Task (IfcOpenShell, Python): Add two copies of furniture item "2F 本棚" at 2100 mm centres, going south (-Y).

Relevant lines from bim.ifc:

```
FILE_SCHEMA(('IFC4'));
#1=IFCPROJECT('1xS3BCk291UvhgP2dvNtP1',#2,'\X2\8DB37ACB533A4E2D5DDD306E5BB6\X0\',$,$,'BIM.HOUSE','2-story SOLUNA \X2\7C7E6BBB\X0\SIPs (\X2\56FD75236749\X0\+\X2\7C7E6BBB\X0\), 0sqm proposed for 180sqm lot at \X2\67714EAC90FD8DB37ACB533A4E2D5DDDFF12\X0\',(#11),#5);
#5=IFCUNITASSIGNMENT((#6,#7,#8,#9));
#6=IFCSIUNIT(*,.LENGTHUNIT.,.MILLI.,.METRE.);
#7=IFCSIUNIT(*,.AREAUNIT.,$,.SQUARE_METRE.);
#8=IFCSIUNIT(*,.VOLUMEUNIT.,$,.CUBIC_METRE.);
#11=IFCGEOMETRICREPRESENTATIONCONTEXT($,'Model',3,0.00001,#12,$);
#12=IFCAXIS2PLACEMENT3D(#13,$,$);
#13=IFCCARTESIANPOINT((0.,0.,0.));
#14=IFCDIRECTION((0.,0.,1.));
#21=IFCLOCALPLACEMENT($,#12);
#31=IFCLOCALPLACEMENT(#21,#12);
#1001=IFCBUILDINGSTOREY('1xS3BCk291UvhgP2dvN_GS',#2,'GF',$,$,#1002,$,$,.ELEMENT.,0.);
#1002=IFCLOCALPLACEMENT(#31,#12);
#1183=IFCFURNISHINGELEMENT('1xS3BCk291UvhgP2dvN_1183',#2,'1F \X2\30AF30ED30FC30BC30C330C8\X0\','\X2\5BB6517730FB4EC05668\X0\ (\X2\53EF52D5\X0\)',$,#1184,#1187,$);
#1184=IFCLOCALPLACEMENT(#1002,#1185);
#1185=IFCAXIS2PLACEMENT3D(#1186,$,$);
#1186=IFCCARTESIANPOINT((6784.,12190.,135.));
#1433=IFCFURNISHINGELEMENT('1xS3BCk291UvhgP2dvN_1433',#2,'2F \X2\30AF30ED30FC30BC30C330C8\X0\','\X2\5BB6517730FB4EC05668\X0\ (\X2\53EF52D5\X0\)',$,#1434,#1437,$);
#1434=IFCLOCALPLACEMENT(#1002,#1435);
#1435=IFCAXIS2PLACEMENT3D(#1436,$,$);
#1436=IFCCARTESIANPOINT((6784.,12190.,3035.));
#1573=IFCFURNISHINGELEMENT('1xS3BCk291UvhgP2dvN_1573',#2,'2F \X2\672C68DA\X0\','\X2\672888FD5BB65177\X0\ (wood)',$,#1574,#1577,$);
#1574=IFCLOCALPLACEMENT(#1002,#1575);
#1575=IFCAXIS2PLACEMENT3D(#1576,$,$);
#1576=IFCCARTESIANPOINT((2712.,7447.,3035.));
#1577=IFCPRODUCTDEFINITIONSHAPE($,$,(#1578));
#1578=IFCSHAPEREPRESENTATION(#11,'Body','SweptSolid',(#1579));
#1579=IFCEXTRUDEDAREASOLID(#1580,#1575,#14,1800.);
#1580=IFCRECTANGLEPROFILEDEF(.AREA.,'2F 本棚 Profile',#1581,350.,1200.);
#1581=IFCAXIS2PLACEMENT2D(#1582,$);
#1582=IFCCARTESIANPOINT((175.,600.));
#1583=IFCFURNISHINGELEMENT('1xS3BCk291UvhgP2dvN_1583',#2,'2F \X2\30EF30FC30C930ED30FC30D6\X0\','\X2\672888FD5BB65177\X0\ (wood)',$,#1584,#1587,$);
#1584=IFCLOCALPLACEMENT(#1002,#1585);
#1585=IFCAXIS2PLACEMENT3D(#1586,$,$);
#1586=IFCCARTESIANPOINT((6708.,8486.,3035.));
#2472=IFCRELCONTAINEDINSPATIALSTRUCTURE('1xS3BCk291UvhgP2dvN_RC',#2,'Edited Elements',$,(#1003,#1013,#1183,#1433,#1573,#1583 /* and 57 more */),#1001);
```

```python
import numpy as np
import ifcopenshell
import ifcopenshell.api.geometry
import ifcopenshell.api.root
import ifcopenshell.util.element
import ifcopenshell.util.placement

model = ifcopenshell.open("bim.ifc")


def reuse_history(source, copy):
    """copy_class also copies each property set's owner history, people and application; keep the originals."""
    for rel in copy.IsDefinedBy:
        if rel.is_a("IfcRelDefinesByProperties") and (history := rel.RelatingPropertyDefinition.OwnerHistory):
            rel.RelatingPropertyDefinition.OwnerHistory = source.OwnerHistory
            ifcopenshell.util.element.remove_deep2(model, history)


source = model.by_id(1573)
base = ifcopenshell.util.placement.get_local_placement(source.ObjectPlacement)
step = np.array([0.0, -1.0, 0.0]) * 2100.0

for i in range(1, 3):
    copy = ifcopenshell.api.root.copy_class(model, product=source)
    copy.Representation = ifcopenshell.util.element.copy_deep(
        model, source.Representation, exclude=["IfcGeometricRepresentationContext", "IfcRepresentationMap"]
    )
    reuse_history(source, copy)
    matrix = base.copy()
    matrix[:3, 3] += i * step
    print("added at", matrix[:3, 3].round(3) + 0.0)
    ifcopenshell.api.geometry.edit_object_placement(model, product=copy, matrix=matrix, is_si=False)

model.write("bim_v2.ifc")
```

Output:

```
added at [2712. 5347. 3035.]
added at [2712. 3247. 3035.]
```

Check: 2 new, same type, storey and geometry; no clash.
